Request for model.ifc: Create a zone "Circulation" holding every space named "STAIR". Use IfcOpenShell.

First a look at what the model holds.

```python
import ifcopenshell

model = ifcopenshell.open("model.ifc")
print(model.schema)
seen = {}
for space in model.by_type("IfcSpace"):
    seen[space.LongName] = seen.get(space.LongName, 0) + 1
for name, count in sorted(seen.items(), key=str):
    print(count, "x", name)
print("zones:", [z.Name for z in model.by_type("IfcZone")][:20])
```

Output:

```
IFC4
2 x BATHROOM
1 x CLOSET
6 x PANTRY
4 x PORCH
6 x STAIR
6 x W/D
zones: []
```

```python
import ifcopenshell
import ifcopenshell.api.group
import ifcopenshell.api.root

model = ifcopenshell.open("model.ifc")

names = {"STAIR"}
spaces = [s for s in model.by_type("IfcSpace") if s.LongName in names]

zone = ifcopenshell.api.root.create_entity(model, ifc_class="IfcZone", name="Circulation")
ifcopenshell.api.group.assign_group(model, products=spaces, group=zone)
print(len(spaces), "spaces in", zone.Name)

model.write("model_updated.ifc")
```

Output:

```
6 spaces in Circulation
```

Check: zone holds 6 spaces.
